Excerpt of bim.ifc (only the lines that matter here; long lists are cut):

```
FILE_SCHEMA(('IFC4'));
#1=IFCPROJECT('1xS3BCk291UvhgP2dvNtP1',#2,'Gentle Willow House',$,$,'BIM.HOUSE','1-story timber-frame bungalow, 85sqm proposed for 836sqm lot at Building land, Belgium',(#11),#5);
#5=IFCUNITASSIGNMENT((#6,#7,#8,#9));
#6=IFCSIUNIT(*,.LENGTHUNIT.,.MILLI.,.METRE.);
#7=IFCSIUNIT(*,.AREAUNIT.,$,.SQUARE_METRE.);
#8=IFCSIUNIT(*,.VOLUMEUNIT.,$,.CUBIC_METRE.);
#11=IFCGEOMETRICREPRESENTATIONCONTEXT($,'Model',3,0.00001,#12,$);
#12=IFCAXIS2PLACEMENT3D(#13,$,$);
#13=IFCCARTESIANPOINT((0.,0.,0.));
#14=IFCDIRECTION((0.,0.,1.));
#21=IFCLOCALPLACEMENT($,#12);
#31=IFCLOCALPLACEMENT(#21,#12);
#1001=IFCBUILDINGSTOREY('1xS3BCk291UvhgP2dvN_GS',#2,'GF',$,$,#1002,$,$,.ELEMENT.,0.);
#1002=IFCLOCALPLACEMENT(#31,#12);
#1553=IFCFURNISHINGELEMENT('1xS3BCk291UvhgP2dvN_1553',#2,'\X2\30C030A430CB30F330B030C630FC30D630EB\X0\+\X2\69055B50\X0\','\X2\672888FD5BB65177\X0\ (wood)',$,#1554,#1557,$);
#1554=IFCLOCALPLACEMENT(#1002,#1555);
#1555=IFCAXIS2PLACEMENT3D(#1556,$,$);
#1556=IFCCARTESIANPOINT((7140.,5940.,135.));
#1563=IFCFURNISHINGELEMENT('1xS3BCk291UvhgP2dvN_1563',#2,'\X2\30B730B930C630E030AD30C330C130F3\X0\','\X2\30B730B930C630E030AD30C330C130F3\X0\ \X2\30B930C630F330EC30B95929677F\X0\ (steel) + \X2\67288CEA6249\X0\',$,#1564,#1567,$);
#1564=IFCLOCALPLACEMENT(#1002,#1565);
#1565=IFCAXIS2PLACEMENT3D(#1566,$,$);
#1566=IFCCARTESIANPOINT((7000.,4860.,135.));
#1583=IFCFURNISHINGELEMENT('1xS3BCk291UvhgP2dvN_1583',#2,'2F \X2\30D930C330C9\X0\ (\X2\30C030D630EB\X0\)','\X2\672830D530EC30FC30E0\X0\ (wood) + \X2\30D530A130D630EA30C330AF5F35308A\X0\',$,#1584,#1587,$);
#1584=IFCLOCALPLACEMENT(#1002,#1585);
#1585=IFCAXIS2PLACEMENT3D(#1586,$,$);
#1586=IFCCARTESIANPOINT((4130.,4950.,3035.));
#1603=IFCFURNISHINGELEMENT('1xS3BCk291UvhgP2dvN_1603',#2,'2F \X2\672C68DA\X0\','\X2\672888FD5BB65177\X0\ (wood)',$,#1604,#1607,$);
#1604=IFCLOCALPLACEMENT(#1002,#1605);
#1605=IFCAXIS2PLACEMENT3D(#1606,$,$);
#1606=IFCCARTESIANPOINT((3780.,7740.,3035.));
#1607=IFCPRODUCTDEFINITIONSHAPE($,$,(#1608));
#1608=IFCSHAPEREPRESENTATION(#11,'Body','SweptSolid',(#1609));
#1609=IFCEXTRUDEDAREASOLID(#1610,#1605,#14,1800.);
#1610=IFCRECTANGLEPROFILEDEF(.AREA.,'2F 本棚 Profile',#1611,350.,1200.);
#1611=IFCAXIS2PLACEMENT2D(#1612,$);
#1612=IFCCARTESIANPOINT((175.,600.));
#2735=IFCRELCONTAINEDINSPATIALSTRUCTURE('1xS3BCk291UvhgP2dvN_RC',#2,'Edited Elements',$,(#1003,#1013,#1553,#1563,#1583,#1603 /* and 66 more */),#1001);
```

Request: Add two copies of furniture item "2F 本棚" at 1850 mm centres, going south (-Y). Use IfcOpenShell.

```python
import numpy as np
import ifcopenshell
import ifcopenshell.api.geometry
import ifcopenshell.api.root
import ifcopenshell.util.element
import ifcopenshell.util.placement

model = ifcopenshell.open("bim.ifc")


def reuse_history(source, copy):
    """copy_class also copies each property set's owner history, people and application; keep the originals."""
    for rel in copy.IsDefinedBy:
        if rel.is_a("IfcRelDefinesByProperties") and (history := rel.RelatingPropertyDefinition.OwnerHistory):
            rel.RelatingPropertyDefinition.OwnerHistory = source.OwnerHistory
            ifcopenshell.util.element.remove_deep2(model, history)


source = model.by_guid("1xS3BCk291UvhgP2dvN_1603")
base = ifcopenshell.util.placement.get_local_placement(source.ObjectPlacement)
step = np.array([0.0, -1.0, 0.0]) * 1850.0

for i in range(1, 3):
    copy = ifcopenshell.api.root.copy_class(model, product=source)
    copy.Representation = ifcopenshell.util.element.copy_deep(
        model, source.Representation, exclude=["IfcGeometricRepresentationContext", "IfcRepresentationMap"]
    )
    reuse_history(source, copy)
    matrix = base.copy()
    matrix[:3, 3] += i * step
    print("added at", matrix[:3, 3].round(3) + 0.0)
    ifcopenshell.api.geometry.edit_object_placement(model, product=copy, matrix=matrix, is_si=False)

model.write("bim_rev.ifc")
```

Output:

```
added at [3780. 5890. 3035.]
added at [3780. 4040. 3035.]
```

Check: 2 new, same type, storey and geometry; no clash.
